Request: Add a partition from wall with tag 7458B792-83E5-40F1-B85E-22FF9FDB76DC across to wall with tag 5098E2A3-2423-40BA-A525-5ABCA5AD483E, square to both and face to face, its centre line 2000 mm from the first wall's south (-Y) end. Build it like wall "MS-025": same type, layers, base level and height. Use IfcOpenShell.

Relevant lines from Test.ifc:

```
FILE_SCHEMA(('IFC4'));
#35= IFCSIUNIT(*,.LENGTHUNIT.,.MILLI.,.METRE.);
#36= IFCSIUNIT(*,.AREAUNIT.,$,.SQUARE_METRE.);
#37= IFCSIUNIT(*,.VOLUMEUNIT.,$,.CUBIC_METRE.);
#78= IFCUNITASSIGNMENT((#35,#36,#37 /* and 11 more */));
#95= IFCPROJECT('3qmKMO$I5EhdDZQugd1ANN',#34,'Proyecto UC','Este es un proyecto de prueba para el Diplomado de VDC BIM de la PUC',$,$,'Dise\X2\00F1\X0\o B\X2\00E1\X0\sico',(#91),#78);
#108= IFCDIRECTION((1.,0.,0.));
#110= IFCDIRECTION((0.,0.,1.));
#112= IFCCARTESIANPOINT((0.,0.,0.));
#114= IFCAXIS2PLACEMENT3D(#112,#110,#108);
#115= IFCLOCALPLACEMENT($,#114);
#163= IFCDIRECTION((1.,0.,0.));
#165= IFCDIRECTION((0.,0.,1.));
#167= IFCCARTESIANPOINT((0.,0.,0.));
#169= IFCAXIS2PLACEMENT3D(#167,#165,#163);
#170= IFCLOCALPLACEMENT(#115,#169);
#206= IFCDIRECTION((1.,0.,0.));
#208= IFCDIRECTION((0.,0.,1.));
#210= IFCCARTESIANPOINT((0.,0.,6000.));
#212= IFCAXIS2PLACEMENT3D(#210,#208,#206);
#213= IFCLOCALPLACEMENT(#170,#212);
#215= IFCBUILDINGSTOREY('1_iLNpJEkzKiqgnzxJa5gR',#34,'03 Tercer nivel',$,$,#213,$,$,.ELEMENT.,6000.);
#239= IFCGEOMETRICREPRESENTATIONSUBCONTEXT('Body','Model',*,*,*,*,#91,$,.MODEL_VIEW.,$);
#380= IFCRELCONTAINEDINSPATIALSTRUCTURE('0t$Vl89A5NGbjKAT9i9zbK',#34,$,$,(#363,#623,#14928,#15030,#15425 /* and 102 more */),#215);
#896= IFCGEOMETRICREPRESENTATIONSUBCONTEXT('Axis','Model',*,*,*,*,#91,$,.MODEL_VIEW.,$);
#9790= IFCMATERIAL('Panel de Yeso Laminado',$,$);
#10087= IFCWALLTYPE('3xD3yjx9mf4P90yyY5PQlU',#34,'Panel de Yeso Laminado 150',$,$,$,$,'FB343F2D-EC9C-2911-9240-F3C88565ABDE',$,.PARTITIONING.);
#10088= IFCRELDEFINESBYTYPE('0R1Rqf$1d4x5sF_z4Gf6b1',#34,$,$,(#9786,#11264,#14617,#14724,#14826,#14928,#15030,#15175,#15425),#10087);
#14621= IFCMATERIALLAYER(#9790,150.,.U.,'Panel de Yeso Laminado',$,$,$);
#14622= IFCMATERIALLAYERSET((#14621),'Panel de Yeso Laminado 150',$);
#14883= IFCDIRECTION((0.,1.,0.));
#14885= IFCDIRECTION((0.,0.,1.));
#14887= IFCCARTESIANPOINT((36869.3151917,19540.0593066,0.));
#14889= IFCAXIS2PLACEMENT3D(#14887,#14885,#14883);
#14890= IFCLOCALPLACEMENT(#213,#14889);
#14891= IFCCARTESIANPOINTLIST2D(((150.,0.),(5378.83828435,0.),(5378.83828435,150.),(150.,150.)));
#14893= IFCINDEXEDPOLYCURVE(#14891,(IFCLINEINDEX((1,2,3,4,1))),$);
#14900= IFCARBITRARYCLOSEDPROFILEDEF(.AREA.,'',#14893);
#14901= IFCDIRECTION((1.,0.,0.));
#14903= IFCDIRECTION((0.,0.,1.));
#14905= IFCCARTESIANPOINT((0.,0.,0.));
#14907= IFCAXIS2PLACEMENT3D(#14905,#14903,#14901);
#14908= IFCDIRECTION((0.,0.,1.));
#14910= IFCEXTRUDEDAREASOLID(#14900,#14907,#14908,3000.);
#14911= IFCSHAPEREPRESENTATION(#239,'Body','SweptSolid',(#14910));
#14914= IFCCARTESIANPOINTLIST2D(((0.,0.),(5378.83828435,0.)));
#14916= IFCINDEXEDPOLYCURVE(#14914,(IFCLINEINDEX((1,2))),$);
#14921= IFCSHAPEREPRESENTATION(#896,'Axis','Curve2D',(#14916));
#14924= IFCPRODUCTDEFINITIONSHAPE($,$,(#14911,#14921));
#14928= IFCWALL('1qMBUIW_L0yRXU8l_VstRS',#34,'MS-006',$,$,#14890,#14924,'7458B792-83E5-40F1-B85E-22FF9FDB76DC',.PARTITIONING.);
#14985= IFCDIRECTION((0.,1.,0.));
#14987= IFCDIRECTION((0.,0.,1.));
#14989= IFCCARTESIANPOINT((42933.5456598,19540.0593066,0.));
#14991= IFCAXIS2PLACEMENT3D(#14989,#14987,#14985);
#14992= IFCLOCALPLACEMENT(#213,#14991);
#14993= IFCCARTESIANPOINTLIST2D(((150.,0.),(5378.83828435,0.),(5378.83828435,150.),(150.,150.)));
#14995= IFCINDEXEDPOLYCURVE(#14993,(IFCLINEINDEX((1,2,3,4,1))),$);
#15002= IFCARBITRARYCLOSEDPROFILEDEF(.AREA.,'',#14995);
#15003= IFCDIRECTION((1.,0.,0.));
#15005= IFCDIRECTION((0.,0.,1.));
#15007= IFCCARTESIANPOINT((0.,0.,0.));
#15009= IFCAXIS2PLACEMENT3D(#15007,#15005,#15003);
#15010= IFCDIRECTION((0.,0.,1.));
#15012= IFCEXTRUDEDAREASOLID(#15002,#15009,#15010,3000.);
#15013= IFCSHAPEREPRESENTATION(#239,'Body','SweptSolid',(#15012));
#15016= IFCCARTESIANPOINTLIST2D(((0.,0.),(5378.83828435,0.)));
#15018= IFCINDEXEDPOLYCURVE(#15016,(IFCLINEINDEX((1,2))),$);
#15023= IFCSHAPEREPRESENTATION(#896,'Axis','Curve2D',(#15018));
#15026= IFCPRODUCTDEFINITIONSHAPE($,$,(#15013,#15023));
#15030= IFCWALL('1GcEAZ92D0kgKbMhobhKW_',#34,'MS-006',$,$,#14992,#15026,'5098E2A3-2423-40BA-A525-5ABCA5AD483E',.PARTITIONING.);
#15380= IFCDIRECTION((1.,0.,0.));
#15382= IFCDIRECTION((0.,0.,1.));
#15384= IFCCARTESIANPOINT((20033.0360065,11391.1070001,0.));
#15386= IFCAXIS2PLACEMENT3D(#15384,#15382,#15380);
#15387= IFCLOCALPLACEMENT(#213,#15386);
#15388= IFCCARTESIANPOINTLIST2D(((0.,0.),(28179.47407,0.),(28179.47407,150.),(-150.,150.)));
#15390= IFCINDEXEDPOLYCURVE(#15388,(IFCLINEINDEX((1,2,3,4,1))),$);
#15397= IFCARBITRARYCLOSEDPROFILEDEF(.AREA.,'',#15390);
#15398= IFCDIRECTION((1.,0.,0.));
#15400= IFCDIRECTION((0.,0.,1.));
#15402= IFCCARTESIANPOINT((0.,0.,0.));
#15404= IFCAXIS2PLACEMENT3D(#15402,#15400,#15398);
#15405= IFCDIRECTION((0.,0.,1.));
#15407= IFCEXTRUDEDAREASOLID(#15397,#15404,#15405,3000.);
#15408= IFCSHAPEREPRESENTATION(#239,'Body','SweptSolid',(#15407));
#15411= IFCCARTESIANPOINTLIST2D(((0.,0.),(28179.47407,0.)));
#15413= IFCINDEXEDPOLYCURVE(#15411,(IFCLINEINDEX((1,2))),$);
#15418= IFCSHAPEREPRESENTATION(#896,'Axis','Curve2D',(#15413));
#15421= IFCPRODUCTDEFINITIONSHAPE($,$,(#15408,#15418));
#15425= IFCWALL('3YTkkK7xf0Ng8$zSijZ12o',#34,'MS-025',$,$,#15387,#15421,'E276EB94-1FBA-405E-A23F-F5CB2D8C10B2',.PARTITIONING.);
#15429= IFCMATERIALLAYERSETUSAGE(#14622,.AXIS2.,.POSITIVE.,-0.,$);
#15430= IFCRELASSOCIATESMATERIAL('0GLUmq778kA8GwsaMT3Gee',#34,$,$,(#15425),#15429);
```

```python
import numpy as np
import ifcopenshell
import ifcopenshell.api.geometry
import ifcopenshell.api.material
import ifcopenshell.api.pset
import ifcopenshell.api.root
import ifcopenshell.api.spatial
import ifcopenshell.api.type
import ifcopenshell.geom
import ifcopenshell.util.element
import ifcopenshell.util.placement
import ifcopenshell.util.representation
import ifcopenshell.util.shape
import ifcopenshell.util.unit

model = ifcopenshell.open("Test.ifc")
unit_scale = ifcopenshell.util.unit.calculate_unit_scale(model)
settings = ifcopenshell.geom.settings()
settings.set("use-world-coords", True)

start_wall = model.by_guid("1qMBUIW_L0yRXU8l_VstRS")
end_wall = model.by_guid("1GcEAZ92D0kgKbMhobhKW_")
like = model.by_id(15425)
matrix = ifcopenshell.util.placement.get_local_placement(start_wall.ObjectPlacement)
matrix[:3, 3] *= unit_scale


def extent(element):
    """Bounding box in the first wall's axes, in metres."""
    shape = ifcopenshell.geom.create_shape(settings, element)
    points = (ifcopenshell.util.shape.get_vertices(shape.geometry) - matrix[:3, 3]) @ matrix[:3, :3]
    return points.min(axis=0), points.max(axis=0)


y_start = extent(start_wall)[0][1]
y_end = extent(end_wall)[1][1]
like_min, like_max = extent(like)
length, height = float(abs(y_end - y_start)), float(like_max[2] - like_min[2])
layer_set = ifcopenshell.util.element.get_material(like, should_skip_usage=True)
thickness = sum(layer.LayerThickness for layer in layer_set.MaterialLayers) * unit_scale

wall = ifcopenshell.api.root.create_entity(model, ifc_class="IfcWall", name="New partition")
storey = ifcopenshell.util.element.get_container(like)
ifcopenshell.api.spatial.assign_container(model, products=[wall], relating_structure=storey)
ifcopenshell.api.type.assign_type(
    model, related_objects=[wall], relating_type=ifcopenshell.util.element.get_type(like), should_map_representations=False
)
rel = ifcopenshell.api.material.assign_material(
    model, products=[wall], type="IfcMaterialLayerSetUsage", material=layer_set
)
rel.RelatingMaterial.OffsetFromReferenceLine = -thickness / 2 / unit_scale
pset = ifcopenshell.api.pset.add_pset(model, product=wall, name="Pset_WallCommon")
ifcopenshell.api.pset.edit_pset(model, pset=pset, properties={"IsExternal": False, "LoadBearing": False})

# The axis runs down the middle of the wall.
axis = ifcopenshell.api.geometry.add_axis_representation(
    model, context=ifcopenshell.util.representation.get_context(model, "Model", "Axis"), axis=[(0.0, 0.0), (length, 0.0)]
)
body = ifcopenshell.api.geometry.add_wall_representation(
    model,
    context=ifcopenshell.util.representation.get_context(model, "Model", "Body", "MODEL_VIEW"),
    length=length,
    height=height,
    thickness=thickness,
    offset=-thickness / 2,
)
for representation in (axis, body):
    ifcopenshell.api.geometry.assign_representation(model, product=wall, representation=representation)

placement = matrix @ ifcopenshell.util.placement.rotation(-90, "Z")
placement[:, 3] = matrix @ np.array([extent(start_wall)[0][0] + 2, y_start, like_min[2], 1.0])
ifcopenshell.api.geometry.edit_object_placement(model, product=wall, matrix=placement)

print(f"partition {length:.3f} m long, {height:.3f} m high, {thickness:.3f} m thick")

model.write("Test_rev.ifc")
```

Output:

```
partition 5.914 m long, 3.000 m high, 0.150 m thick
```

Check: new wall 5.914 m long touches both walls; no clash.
